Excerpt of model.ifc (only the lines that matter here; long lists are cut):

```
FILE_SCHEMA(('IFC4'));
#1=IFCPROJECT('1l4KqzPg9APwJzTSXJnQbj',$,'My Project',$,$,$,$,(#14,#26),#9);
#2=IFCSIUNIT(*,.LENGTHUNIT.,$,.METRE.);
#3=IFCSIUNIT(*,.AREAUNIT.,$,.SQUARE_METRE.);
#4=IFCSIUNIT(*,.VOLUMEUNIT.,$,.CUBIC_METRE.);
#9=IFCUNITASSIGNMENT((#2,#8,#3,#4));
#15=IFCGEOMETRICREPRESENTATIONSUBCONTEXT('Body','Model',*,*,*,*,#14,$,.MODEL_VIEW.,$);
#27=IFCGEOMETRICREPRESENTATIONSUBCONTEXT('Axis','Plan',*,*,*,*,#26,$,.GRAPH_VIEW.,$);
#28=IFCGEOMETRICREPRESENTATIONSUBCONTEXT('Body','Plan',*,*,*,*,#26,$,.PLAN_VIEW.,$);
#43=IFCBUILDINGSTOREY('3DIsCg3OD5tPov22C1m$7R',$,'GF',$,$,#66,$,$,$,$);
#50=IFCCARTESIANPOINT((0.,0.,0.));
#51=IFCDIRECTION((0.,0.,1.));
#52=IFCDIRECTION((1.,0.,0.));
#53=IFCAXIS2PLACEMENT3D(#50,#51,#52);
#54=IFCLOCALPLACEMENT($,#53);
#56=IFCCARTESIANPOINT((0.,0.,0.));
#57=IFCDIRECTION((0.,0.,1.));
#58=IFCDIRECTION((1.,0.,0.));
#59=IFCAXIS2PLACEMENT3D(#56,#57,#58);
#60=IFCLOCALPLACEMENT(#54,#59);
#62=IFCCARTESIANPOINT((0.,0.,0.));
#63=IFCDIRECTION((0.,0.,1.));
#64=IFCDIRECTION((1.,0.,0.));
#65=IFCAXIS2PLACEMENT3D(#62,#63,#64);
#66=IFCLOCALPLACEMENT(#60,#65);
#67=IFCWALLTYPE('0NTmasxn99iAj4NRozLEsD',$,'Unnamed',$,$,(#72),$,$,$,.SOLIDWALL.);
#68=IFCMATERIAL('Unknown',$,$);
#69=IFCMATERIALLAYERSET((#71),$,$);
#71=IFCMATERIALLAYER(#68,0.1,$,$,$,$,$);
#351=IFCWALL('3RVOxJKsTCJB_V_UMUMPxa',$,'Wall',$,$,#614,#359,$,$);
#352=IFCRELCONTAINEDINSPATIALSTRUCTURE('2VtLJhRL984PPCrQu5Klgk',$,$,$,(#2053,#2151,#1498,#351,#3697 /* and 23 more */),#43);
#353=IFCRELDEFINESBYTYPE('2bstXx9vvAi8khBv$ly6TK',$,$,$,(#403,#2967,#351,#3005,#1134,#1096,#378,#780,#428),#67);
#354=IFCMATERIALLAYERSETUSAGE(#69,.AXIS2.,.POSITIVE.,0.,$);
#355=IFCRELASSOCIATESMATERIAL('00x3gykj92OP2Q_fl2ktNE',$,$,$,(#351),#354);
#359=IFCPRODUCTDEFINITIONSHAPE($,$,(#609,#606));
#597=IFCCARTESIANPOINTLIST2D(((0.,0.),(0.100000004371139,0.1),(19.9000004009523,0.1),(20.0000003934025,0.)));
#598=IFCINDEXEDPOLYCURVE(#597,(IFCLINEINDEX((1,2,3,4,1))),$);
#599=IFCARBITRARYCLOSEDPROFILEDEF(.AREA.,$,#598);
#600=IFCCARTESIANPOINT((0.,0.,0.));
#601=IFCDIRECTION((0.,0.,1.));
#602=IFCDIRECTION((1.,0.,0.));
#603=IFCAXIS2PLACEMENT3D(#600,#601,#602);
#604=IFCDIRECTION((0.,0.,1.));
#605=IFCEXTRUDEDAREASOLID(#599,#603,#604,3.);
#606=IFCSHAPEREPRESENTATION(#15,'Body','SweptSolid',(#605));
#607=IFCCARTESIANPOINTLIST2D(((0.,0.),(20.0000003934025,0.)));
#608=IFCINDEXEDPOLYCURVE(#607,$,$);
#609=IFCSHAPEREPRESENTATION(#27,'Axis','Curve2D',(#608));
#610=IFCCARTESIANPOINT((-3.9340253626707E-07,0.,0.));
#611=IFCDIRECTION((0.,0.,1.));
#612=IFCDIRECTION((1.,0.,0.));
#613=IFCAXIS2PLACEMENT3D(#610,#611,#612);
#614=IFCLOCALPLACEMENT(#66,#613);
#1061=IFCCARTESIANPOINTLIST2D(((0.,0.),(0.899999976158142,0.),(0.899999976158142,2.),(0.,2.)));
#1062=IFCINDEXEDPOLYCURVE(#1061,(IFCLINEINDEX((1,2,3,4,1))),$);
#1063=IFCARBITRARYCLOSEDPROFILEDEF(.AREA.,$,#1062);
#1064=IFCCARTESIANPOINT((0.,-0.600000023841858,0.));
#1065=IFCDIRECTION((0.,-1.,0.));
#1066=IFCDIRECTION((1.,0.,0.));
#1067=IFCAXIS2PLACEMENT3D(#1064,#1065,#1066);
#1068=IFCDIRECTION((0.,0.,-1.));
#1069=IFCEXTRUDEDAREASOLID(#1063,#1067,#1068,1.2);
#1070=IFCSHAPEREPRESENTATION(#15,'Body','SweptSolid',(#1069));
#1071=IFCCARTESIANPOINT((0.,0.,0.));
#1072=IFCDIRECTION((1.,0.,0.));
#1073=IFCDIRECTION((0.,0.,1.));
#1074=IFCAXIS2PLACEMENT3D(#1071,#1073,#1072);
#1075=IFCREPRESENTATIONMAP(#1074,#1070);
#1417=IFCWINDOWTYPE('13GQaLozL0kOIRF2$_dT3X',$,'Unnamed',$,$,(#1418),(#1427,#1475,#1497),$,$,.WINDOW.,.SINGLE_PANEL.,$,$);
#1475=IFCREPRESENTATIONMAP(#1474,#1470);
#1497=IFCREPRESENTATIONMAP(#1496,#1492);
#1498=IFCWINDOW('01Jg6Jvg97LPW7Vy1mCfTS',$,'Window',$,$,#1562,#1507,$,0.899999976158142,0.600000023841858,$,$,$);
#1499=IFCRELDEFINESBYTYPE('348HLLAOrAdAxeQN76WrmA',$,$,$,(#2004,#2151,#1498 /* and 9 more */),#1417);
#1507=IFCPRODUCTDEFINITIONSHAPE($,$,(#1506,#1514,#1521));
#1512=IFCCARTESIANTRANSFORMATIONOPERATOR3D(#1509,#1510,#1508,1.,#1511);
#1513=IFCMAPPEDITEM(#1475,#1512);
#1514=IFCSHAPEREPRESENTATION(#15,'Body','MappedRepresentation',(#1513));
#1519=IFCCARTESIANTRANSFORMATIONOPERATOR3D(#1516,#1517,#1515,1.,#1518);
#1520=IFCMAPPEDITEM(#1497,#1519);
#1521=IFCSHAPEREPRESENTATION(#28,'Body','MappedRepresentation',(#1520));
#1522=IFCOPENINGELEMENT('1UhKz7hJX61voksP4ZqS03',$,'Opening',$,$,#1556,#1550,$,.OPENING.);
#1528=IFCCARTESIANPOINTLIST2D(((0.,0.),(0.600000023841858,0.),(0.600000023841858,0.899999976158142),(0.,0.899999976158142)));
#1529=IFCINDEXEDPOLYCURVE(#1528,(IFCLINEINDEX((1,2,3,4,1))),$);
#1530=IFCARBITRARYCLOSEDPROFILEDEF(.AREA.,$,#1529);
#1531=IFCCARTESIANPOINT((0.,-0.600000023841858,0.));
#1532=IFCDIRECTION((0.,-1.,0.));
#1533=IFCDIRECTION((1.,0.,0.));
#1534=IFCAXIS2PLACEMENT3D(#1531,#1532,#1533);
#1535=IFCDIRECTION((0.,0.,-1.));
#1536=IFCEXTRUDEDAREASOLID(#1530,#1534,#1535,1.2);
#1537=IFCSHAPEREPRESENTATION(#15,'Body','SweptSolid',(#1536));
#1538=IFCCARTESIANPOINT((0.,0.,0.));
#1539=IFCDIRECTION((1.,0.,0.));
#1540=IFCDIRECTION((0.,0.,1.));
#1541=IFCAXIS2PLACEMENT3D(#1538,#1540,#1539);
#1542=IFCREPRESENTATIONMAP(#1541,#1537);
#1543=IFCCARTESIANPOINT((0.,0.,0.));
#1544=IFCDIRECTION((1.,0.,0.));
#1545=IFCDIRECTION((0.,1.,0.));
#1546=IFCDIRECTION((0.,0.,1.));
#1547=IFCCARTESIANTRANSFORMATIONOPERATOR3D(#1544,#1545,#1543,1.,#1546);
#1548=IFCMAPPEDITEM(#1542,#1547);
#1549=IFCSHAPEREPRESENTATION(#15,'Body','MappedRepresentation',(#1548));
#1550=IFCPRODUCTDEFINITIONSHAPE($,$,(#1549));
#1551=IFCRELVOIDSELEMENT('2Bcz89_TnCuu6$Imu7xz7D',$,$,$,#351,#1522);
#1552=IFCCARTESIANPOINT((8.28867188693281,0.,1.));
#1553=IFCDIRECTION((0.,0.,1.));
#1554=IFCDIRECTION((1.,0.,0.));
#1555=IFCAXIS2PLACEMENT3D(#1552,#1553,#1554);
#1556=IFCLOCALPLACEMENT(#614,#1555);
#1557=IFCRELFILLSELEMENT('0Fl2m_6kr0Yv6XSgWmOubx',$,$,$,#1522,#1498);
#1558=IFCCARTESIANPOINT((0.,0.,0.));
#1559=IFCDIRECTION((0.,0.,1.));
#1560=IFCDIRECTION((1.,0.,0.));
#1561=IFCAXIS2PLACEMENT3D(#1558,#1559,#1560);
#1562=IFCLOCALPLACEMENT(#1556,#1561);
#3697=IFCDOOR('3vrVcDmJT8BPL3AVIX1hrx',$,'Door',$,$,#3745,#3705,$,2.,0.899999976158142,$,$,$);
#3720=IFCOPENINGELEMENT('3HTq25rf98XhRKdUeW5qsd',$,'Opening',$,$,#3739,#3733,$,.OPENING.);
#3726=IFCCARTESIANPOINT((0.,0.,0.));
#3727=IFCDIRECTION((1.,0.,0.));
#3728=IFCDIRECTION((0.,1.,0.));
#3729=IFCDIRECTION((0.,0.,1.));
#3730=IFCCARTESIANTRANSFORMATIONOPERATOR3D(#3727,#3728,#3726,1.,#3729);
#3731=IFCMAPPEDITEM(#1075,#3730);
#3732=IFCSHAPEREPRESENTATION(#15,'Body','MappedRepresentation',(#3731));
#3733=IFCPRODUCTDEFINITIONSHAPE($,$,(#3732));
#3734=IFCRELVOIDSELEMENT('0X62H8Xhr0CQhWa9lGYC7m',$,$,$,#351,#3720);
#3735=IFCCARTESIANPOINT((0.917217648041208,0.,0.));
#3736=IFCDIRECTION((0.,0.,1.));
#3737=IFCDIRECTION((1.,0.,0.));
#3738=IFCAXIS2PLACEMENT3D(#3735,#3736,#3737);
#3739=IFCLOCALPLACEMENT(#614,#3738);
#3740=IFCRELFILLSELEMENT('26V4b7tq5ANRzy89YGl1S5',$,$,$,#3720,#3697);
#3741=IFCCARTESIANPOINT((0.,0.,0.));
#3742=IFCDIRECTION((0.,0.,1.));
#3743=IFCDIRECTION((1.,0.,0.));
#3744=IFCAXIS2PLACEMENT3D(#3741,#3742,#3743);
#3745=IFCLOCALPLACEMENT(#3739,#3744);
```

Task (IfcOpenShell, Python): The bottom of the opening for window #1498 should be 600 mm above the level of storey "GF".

```python
import numpy as np
import ifcopenshell
import ifcopenshell.api.geometry
import ifcopenshell.geom
import ifcopenshell.util.element
import ifcopenshell.util.placement
import ifcopenshell.util.shape
import ifcopenshell.util.unit

model = ifcopenshell.open("model.ifc")
unit_scale = ifcopenshell.util.unit.calculate_unit_scale(model)

window = model.by_id(1498)
opening = window.FillsVoids[0].RelatingOpeningElement
storey = ifcopenshell.util.element.get_container(window, ifc_class="IfcBuildingStorey")
level = ifcopenshell.util.placement.get_local_placement(storey.ObjectPlacement)[2, 3]

# The opening's origin need not be at the sill, so measure its lowest point.
shape = ifcopenshell.geom.create_shape(ifcopenshell.geom.settings(), opening)
bottom = ifcopenshell.util.shape.get_shape_bottom_elevation(shape, shape.geometry) / unit_scale
dz = level + 0.6 / unit_scale - bottom

shift = np.array([0.0, 0.0, dz])
# The window is placed relative to its opening, so it follows when the opening moves.
matrix = ifcopenshell.util.placement.get_local_placement(opening.ObjectPlacement)
matrix[:3, 3] += shift
ifcopenshell.api.geometry.edit_object_placement(
    model, product=opening, matrix=matrix, is_si=False, should_transform_children=True
)

print(f"moved by {dz * unit_scale:+.3f} m")

model.write("model_edited.ifc")
```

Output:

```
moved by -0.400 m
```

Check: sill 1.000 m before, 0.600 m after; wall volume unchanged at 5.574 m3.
